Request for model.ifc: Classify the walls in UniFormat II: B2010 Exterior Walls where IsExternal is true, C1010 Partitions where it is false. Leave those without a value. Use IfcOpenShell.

First a look at what the model holds.

```python
import ifcopenshell
import ifcopenshell.util.element

model = ifcopenshell.open("model.ifc")
print(model.schema)
print("classifications:", [c.Name for c in model.by_type("IfcClassification")])
values = [ifcopenshell.util.element.get_pset(e, "Pset_WallCommon", "IsExternal") for e in model.by_type("IfcWall")]
for value in (True, False, None):
    print("IsExternal", value, values.count(value))
```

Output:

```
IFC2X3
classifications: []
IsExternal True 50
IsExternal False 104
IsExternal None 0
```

```python
import ifcopenshell
import ifcopenshell.api.classification
import ifcopenshell.util.element

model = ifcopenshell.open("model.ifc")

# IFC2X3 requires Source and Edition and has no link from the project to the system.
system = model.create_entity("IfcClassification", Source="ASTM", Edition="E1557", Name="UniFormat II")

walls = model.by_type("IfcWall")
external = {e: ifcopenshell.util.element.get_pset(e, "Pset_WallCommon", "IsExternal") for e in walls}
for flag, code, name in ((True, "B2010", "Exterior Walls"), (False, "C1010", "Partitions")):
    products = [e for e in walls if external[e] is flag]
    ifcopenshell.api.classification.add_reference(
        model, products=products, classification=system, identification=code, name=name
    )
    print(code, len(products))

model.write("model-out.ifc")
```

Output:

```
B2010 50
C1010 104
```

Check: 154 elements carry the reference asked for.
